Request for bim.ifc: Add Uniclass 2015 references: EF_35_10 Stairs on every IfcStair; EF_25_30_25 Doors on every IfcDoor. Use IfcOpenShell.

First a look at what the model holds.

```python
import ifcopenshell

model = ifcopenshell.open("bim.ifc")
print(model.schema)
print("classifications:", [c.Name for c in model.by_type("IfcClassification")])
for ifc_class in ("IfcDoor", "IfcRoof", "IfcStair", "IfcWall", "IfcWindow"):
    print(ifc_class, len(model.by_type(ifc_class)))
```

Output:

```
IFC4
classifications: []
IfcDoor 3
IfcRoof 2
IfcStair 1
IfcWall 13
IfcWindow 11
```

```python
import ifcopenshell
import ifcopenshell.api.classification

model = ifcopenshell.open("bim.ifc")

system = ifcopenshell.api.classification.add_classification(model, classification="Uniclass 2015")

codes = {
    "IfcStair": ("EF_35_10", "Stairs"),
    "IfcDoor": ("EF_25_30_25", "Doors"),
}
for ifc_class, (code, name) in codes.items():
    products = model.by_type(ifc_class)
    ifcopenshell.api.classification.add_reference(
        model, products=products, classification=system, identification=code, name=name
    )
    print(code, len(products))

model.write("bim_v2.ifc")
```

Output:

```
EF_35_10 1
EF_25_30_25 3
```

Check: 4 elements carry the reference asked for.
